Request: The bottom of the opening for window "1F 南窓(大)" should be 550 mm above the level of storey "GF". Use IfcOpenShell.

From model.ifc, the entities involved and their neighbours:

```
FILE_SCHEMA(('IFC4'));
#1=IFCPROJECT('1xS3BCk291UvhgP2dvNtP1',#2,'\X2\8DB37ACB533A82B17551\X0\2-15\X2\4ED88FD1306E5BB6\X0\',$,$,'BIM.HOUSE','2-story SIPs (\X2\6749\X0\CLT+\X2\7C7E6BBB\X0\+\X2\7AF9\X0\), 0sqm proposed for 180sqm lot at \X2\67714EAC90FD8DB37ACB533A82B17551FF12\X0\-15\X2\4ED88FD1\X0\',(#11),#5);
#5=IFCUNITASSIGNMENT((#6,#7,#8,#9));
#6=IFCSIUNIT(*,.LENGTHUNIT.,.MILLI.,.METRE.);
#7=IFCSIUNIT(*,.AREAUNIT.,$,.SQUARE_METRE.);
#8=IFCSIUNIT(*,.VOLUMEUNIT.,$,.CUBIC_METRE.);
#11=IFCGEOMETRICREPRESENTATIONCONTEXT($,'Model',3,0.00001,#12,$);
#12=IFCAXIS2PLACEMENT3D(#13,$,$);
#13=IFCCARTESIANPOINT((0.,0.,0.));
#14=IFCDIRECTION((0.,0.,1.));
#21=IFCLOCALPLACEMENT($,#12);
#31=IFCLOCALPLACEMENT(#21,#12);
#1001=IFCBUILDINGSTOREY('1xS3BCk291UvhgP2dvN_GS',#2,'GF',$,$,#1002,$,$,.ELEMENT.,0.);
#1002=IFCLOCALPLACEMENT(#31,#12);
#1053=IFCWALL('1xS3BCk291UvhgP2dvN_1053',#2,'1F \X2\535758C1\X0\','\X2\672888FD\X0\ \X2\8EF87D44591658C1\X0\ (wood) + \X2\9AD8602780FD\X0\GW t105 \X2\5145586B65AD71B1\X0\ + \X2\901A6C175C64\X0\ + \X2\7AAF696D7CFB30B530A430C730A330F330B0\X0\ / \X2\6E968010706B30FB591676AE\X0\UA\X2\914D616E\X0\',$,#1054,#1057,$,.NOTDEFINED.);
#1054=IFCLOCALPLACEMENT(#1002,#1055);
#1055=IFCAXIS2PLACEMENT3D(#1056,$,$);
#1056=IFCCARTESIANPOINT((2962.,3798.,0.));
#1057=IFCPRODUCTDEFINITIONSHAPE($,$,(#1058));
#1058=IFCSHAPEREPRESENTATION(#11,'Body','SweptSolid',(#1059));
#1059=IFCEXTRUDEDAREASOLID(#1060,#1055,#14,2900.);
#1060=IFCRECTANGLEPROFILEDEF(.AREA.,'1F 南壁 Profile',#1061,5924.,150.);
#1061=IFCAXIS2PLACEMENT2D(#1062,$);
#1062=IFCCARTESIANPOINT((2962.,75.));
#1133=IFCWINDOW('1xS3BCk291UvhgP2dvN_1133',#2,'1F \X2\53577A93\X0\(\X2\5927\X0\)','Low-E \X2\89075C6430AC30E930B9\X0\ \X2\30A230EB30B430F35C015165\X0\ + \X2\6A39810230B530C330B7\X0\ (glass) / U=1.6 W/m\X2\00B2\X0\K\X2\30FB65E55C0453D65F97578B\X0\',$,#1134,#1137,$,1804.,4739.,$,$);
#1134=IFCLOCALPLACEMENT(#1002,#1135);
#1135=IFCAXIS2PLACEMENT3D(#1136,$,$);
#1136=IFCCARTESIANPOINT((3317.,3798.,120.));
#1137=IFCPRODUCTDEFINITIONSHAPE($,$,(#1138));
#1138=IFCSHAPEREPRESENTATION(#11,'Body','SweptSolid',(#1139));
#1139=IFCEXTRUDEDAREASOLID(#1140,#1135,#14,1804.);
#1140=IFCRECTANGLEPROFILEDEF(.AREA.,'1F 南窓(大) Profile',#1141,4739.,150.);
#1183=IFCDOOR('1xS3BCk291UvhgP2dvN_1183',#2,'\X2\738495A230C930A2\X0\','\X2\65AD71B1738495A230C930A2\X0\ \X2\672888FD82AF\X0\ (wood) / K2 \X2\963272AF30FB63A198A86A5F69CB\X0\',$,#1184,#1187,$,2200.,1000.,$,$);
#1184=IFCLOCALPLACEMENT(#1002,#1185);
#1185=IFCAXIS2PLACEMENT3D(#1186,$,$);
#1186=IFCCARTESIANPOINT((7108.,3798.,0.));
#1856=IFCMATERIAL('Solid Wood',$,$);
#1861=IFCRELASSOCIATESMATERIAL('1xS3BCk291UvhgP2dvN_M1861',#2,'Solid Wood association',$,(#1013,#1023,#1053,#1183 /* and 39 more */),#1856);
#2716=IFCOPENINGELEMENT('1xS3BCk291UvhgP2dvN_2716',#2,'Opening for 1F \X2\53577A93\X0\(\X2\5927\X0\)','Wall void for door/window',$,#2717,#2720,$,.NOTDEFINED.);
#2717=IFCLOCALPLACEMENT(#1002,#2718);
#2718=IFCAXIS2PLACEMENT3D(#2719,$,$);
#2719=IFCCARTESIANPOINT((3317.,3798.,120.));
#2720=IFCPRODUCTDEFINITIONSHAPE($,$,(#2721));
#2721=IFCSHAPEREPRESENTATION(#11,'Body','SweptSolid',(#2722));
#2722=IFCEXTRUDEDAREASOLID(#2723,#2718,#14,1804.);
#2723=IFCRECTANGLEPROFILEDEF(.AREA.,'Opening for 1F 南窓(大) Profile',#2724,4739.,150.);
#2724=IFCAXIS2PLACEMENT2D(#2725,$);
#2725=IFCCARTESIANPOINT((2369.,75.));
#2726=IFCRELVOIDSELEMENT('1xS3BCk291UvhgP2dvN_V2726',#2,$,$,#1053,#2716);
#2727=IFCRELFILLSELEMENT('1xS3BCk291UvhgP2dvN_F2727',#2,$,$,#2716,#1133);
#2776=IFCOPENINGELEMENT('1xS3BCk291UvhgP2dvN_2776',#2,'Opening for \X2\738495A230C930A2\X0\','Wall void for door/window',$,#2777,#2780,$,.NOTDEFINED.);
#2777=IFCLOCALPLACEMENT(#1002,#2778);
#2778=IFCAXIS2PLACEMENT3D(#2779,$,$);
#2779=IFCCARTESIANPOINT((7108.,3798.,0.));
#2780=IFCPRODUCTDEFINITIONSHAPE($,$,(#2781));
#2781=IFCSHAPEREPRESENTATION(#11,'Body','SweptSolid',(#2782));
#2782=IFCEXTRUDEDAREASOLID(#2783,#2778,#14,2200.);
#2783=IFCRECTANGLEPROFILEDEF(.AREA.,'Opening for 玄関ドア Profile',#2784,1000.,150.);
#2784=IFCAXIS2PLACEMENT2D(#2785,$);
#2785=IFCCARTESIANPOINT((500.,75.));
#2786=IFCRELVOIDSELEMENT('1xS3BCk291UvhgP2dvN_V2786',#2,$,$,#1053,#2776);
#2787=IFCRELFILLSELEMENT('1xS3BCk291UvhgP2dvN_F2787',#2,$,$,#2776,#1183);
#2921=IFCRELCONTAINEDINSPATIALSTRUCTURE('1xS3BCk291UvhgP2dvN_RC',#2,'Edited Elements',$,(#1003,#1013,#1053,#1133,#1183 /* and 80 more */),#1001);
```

```python
import numpy as np
import ifcopenshell
import ifcopenshell.api.geometry
import ifcopenshell.geom
import ifcopenshell.util.element
import ifcopenshell.util.placement
import ifcopenshell.util.shape
import ifcopenshell.util.unit

model = ifcopenshell.open("model.ifc")
unit_scale = ifcopenshell.util.unit.calculate_unit_scale(model)

window = model.by_guid("1xS3BCk291UvhgP2dvN_1133")
opening = window.FillsVoids[0].RelatingOpeningElement
storey = ifcopenshell.util.element.get_container(window, ifc_class="IfcBuildingStorey")
level = ifcopenshell.util.placement.get_local_placement(storey.ObjectPlacement)[2, 3]

# The opening's origin need not be at the sill, so measure its lowest point.
shape = ifcopenshell.geom.create_shape(ifcopenshell.geom.settings(), opening)
bottom = ifcopenshell.util.shape.get_shape_bottom_elevation(shape, shape.geometry) / unit_scale
dz = level + 0.55 / unit_scale - bottom

shift = np.array([0.0, 0.0, dz])
# The window is not placed relative to its opening, so move both.
for product in (opening, window):
    matrix = ifcopenshell.util.placement.get_local_placement(product.ObjectPlacement)
    matrix[:3, 3] += shift
    ifcopenshell.api.geometry.edit_object_placement(model, product=product, matrix=matrix, is_si=False)

print(f"moved by {dz * unit_scale:+.3f} m")

model.write("model-out.ifc")
```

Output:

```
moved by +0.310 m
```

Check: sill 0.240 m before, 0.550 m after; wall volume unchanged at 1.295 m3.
